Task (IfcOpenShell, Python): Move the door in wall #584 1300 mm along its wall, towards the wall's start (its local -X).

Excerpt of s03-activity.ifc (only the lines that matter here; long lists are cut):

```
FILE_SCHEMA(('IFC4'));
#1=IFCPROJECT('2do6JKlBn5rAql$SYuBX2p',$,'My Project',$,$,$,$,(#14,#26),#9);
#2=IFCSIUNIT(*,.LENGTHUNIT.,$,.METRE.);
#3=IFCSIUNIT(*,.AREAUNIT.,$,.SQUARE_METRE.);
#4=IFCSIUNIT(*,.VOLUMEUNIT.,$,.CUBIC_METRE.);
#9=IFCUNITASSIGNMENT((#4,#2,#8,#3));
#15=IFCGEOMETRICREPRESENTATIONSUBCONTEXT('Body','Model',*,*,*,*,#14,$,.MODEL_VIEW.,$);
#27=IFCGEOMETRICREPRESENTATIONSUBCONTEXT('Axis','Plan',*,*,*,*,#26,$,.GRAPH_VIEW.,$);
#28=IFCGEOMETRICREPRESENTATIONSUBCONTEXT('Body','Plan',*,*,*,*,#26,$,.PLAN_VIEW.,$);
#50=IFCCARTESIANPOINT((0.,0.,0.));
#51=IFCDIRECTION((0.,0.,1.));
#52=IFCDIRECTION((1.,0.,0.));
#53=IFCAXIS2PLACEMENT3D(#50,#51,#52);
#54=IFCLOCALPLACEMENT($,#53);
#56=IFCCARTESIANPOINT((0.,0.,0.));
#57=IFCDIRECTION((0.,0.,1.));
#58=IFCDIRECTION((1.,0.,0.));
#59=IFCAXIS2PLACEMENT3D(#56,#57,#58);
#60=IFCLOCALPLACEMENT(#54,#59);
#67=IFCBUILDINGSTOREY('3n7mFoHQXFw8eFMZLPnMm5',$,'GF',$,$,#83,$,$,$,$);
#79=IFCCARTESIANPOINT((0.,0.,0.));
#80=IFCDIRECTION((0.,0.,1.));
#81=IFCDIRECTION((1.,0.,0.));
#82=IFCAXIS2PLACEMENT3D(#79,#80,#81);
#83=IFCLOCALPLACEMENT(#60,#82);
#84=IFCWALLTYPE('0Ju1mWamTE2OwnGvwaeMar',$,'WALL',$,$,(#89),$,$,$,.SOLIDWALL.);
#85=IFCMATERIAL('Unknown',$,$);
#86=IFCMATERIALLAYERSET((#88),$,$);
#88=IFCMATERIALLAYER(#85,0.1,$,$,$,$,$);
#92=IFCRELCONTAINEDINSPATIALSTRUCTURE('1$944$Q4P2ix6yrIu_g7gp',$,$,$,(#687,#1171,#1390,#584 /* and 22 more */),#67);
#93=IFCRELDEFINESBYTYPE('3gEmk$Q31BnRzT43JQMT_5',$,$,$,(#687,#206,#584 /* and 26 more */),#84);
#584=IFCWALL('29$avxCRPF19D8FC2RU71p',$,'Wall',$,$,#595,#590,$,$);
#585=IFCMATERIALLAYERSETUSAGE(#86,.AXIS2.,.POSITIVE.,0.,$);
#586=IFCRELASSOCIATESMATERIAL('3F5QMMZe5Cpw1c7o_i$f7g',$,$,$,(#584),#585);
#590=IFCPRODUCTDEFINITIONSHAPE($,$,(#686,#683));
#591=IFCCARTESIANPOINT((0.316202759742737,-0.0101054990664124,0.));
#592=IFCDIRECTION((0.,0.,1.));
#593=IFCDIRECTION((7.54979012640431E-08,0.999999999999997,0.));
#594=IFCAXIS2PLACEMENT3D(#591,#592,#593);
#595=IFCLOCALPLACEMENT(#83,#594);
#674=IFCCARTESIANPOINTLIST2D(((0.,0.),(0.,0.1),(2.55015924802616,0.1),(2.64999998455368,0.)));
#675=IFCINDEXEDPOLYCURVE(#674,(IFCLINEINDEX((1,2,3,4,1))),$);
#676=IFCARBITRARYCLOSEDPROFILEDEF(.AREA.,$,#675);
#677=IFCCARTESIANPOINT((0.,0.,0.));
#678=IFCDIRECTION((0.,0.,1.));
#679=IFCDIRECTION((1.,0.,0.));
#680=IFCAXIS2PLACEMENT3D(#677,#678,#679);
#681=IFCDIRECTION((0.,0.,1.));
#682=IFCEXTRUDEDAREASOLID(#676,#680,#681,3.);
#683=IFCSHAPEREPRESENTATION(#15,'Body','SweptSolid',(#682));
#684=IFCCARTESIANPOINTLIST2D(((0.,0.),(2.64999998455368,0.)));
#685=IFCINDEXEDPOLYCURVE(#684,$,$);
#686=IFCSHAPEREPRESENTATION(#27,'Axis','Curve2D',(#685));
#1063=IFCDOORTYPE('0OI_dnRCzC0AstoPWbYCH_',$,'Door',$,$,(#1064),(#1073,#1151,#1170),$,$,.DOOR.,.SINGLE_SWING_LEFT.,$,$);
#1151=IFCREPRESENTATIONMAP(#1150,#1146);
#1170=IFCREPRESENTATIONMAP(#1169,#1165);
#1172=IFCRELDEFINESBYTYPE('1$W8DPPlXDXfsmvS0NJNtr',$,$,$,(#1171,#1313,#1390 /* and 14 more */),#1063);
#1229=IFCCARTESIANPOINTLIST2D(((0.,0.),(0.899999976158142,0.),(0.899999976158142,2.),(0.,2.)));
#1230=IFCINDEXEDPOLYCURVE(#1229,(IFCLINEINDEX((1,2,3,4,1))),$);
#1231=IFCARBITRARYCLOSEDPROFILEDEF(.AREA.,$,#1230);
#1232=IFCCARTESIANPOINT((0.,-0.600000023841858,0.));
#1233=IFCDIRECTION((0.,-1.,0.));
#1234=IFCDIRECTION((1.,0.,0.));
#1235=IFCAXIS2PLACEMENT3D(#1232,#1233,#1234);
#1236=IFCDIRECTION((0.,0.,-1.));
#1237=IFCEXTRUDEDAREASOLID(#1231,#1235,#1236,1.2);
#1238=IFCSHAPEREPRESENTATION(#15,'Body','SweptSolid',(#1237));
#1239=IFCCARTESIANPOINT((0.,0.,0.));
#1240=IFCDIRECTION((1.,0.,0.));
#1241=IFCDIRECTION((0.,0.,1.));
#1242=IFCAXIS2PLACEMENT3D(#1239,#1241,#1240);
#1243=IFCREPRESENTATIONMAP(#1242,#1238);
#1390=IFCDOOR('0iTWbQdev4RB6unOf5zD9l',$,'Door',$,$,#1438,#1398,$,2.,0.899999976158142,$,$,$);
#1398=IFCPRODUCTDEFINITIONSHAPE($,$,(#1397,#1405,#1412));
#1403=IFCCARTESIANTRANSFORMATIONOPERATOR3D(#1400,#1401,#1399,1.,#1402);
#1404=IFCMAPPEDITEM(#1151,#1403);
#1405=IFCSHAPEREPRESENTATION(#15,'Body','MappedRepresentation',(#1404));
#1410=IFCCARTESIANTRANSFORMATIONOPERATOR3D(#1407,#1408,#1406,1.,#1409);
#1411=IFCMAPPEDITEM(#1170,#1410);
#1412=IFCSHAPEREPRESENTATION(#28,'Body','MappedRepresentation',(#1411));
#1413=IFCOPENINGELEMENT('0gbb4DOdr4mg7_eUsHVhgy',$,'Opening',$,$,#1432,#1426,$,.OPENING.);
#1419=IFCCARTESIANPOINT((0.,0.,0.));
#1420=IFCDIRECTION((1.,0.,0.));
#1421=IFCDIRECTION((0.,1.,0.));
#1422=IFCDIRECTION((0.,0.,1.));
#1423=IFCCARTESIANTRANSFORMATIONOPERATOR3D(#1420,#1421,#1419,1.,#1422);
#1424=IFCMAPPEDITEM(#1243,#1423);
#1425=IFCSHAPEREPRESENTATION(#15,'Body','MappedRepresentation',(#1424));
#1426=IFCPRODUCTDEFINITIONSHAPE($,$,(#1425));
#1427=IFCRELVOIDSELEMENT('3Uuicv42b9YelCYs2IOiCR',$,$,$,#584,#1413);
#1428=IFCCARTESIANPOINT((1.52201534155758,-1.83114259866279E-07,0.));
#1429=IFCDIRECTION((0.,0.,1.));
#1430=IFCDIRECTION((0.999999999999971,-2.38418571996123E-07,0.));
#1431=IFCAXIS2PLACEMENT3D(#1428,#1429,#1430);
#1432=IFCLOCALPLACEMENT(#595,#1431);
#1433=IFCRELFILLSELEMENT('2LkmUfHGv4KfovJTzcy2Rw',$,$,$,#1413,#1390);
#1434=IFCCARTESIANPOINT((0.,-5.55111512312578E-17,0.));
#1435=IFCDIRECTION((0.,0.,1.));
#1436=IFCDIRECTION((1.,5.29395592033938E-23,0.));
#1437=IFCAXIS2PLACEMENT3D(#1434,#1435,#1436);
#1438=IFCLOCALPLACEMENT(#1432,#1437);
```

```python
import ifcopenshell
import ifcopenshell.api.geometry
import ifcopenshell.util.placement
import ifcopenshell.util.unit

model = ifcopenshell.open("s03-activity.ifc")
unit_scale = ifcopenshell.util.unit.calculate_unit_scale(model)

door = model.by_id(1390)
opening = door.FillsVoids[0].RelatingOpeningElement
wall = opening.VoidsElements[0].RelatingBuildingElement

wall_matrix = ifcopenshell.util.placement.get_local_placement(wall.ObjectPlacement)
shift = wall_matrix[:3, 0] * -1.3 / unit_scale
before = ifcopenshell.util.placement.get_local_placement(door.ObjectPlacement)[:3, 3].copy()

# The door is placed relative to its opening, so it follows when the opening moves.
matrix = ifcopenshell.util.placement.get_local_placement(opening.ObjectPlacement)
matrix[:3, 3] += shift
ifcopenshell.api.geometry.edit_object_placement(
    model, product=opening, matrix=matrix, is_si=False, should_transform_children=True
)

after = ifcopenshell.util.placement.get_local_placement(door.ObjectPlacement)[:3, 3]
print("door moved by", (after - before).round(3) + 0.0)

model.write("s03-activity-out.ifc")
```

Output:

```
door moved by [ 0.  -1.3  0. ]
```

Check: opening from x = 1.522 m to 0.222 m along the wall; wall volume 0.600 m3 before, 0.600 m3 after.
